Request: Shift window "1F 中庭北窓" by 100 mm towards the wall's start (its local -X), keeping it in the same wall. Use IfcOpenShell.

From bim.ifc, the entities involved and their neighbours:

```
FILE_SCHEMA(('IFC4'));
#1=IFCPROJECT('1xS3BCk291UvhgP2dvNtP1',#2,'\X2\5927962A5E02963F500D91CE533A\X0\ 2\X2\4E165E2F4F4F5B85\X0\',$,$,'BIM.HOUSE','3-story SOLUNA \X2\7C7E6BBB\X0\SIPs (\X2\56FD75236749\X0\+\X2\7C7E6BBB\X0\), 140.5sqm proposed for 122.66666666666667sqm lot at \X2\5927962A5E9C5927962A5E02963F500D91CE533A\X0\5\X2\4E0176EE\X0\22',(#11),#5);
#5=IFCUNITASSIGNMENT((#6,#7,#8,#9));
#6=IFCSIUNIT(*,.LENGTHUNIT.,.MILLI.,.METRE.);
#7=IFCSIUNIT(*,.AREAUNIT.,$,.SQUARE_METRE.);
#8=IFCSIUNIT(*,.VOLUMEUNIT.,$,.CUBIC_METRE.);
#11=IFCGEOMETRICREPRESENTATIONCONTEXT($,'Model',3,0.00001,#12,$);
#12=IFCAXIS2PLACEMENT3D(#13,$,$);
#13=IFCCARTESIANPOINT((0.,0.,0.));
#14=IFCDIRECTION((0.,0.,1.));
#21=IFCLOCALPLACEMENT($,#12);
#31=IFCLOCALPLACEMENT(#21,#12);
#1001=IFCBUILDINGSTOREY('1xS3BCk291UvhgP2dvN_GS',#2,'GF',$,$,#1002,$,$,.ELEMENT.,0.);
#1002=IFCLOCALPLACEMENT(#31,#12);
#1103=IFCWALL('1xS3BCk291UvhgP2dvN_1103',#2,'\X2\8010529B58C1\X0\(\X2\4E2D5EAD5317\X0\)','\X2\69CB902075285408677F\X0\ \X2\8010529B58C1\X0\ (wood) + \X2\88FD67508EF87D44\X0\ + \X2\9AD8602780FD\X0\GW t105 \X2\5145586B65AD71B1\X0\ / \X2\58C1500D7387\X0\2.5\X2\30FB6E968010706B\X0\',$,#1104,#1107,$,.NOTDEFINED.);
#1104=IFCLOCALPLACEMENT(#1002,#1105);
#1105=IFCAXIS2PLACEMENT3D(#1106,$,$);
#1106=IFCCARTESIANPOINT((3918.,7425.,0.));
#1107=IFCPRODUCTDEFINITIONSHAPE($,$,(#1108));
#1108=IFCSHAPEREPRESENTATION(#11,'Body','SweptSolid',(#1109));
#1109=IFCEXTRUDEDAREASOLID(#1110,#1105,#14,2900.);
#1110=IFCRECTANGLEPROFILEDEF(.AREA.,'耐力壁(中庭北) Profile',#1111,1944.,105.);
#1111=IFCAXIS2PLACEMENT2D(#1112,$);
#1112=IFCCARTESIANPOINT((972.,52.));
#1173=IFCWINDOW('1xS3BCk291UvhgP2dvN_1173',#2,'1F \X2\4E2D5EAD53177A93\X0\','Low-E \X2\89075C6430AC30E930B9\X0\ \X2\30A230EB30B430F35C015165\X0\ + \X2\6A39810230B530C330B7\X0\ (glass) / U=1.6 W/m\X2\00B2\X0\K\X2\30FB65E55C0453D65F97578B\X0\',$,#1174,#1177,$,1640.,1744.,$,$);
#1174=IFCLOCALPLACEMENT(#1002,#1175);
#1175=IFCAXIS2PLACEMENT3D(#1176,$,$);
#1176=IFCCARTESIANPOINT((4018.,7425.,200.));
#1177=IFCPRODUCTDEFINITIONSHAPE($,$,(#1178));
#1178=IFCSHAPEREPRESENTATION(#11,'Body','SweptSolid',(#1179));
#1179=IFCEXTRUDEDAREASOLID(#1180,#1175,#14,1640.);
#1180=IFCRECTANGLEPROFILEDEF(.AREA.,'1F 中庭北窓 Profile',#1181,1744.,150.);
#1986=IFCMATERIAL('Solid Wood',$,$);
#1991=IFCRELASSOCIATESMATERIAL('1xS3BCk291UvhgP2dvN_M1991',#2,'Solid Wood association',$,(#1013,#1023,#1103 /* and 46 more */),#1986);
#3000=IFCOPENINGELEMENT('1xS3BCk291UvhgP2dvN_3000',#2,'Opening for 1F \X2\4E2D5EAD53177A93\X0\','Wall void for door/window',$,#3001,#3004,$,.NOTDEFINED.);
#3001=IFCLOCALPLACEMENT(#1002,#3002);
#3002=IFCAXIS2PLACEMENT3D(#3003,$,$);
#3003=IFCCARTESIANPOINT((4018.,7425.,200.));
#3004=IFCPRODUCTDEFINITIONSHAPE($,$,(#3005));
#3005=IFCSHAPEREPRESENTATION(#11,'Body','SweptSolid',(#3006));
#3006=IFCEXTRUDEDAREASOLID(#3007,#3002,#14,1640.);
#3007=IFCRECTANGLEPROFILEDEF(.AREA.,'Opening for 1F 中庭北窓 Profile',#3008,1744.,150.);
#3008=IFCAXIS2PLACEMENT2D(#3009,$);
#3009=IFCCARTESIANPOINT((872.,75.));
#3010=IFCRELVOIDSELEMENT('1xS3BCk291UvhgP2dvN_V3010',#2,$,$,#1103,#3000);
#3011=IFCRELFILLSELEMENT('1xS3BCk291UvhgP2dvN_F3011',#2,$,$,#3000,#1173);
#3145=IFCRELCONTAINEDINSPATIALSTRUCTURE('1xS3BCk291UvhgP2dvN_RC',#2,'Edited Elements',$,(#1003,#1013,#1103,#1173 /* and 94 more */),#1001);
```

```python
import ifcopenshell
import ifcopenshell.api.geometry
import ifcopenshell.util.placement

model = ifcopenshell.open("bim.ifc")

window = model.by_guid("1xS3BCk291UvhgP2dvN_1173")
opening = window.FillsVoids[0].RelatingOpeningElement
wall = opening.VoidsElements[0].RelatingBuildingElement

wall_matrix = ifcopenshell.util.placement.get_local_placement(wall.ObjectPlacement)
shift = wall_matrix[:3, 0] * -100.0
before = ifcopenshell.util.placement.get_local_placement(window.ObjectPlacement)[:3, 3].copy()

# The window is not placed relative to its opening, so move both.
for product in (opening, window):
    matrix = ifcopenshell.util.placement.get_local_placement(product.ObjectPlacement)
    matrix[:3, 3] += shift
    ifcopenshell.api.geometry.edit_object_placement(model, product=product, matrix=matrix, is_si=False)

after = ifcopenshell.util.placement.get_local_placement(window.ObjectPlacement)[:3, 3]
print("window moved by", (after - before).round(3) + 0.0)

model.write("bim_rev.ifc")
```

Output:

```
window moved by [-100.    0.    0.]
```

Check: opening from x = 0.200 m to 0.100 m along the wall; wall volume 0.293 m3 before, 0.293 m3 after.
